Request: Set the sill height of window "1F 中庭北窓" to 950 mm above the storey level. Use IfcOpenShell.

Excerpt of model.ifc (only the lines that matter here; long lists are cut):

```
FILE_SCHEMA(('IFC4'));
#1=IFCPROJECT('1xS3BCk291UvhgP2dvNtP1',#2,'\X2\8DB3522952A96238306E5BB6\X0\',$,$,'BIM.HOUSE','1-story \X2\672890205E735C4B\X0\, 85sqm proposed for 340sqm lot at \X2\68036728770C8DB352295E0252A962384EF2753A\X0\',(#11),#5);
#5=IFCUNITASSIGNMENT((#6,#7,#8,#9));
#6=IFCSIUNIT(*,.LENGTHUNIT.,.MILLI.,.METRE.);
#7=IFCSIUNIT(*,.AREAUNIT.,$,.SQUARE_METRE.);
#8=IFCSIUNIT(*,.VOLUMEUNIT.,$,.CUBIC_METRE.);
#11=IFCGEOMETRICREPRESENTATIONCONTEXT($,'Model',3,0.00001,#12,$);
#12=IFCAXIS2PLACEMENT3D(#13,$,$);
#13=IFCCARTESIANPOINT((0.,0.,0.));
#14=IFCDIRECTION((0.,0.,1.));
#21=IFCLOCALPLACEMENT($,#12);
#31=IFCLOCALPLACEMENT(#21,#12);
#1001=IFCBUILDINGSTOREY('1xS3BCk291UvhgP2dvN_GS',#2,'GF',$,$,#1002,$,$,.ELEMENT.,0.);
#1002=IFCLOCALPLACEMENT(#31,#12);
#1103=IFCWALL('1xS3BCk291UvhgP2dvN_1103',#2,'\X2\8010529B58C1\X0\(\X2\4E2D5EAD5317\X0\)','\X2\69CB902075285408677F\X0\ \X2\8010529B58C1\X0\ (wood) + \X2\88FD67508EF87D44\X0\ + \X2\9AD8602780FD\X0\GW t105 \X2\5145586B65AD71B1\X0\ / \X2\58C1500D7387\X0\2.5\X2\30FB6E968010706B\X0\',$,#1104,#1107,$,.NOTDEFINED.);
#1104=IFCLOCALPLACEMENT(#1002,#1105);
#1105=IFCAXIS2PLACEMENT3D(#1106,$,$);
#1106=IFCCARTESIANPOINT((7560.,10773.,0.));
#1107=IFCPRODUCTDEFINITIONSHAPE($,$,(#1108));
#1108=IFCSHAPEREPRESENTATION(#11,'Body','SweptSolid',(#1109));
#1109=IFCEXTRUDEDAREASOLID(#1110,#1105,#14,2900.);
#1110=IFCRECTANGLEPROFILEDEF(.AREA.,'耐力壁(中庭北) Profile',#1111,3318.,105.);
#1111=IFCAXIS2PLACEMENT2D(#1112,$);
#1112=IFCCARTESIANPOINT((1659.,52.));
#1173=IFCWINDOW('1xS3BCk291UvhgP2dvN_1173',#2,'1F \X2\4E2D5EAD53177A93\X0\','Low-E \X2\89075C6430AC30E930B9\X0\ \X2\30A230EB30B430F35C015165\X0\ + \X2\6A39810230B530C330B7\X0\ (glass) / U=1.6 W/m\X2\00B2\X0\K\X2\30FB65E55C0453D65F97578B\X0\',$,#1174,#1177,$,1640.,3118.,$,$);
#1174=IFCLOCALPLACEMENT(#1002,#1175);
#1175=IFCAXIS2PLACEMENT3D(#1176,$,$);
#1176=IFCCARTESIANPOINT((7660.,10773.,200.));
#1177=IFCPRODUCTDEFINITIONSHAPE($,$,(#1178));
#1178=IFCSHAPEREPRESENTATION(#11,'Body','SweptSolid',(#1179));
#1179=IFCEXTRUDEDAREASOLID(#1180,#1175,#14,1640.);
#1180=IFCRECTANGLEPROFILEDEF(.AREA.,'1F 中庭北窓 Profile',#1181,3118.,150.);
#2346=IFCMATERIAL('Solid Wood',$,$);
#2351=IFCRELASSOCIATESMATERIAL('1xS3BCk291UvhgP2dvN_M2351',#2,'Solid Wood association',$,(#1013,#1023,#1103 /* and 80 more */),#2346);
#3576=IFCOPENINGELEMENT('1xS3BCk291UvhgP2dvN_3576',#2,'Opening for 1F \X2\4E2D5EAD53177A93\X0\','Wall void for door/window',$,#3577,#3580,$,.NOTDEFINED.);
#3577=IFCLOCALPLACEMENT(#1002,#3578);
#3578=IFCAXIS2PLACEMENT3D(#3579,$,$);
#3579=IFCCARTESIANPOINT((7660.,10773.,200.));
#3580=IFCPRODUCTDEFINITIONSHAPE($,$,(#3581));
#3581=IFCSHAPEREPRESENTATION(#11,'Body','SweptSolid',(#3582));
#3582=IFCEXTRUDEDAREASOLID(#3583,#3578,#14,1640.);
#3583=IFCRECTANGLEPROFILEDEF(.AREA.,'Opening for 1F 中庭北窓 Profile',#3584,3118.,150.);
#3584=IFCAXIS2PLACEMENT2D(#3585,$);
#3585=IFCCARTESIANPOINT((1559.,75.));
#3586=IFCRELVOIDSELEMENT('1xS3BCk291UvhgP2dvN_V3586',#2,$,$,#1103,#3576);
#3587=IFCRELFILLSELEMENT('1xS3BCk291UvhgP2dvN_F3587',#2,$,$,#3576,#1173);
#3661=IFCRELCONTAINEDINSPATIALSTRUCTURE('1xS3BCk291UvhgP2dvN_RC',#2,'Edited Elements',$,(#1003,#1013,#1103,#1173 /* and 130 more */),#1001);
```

```python
import numpy as np
import ifcopenshell
import ifcopenshell.api.geometry
import ifcopenshell.geom
import ifcopenshell.util.element
import ifcopenshell.util.placement
import ifcopenshell.util.shape
import ifcopenshell.util.unit

model = ifcopenshell.open("model.ifc")
unit_scale = ifcopenshell.util.unit.calculate_unit_scale(model)

window = model.by_guid("1xS3BCk291UvhgP2dvN_1173")
opening = window.FillsVoids[0].RelatingOpeningElement
storey = ifcopenshell.util.element.get_container(window, ifc_class="IfcBuildingStorey")
level = ifcopenshell.util.placement.get_local_placement(storey.ObjectPlacement)[2, 3]

# The opening's origin need not be at the sill, so measure its lowest point.
shape = ifcopenshell.geom.create_shape(ifcopenshell.geom.settings(), opening)
bottom = ifcopenshell.util.shape.get_shape_bottom_elevation(shape, shape.geometry) / unit_scale
dz = level + 0.95 / unit_scale - bottom

shift = np.array([0.0, 0.0, dz])
# The window is not placed relative to its opening, so move both.
for product in (opening, window):
    matrix = ifcopenshell.util.placement.get_local_placement(product.ObjectPlacement)
    matrix[:3, 3] += shift
    ifcopenshell.api.geometry.edit_object_placement(model, product=product, matrix=matrix, is_si=False)

print(f"moved by {dz * unit_scale:+.3f} m")

model.write("model_rev.ifc")
```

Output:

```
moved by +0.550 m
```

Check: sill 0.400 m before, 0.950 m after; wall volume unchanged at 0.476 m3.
